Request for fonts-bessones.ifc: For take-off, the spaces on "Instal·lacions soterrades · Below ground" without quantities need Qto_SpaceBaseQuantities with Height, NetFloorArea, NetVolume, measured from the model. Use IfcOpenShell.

First a look at what the model holds.

```python
import ifcopenshell
import ifcopenshell.util.element
import ifcopenshell.util.unit

model = ifcopenshell.open("fonts-bessones.ifc")
print(model.schema)
for unit_type in ("LENGTHUNIT", "AREAUNIT", "VOLUMEUNIT"):
    print(unit_type, ifcopenshell.util.unit.calculate_unit_scale(model, unit_type))
storey = next(s for s in model.by_type("IfcBuildingStorey") if s.Name == "Instal·lacions soterrades · Below ground")
spaces = [e for e in ifcopenshell.util.element.get_decomposition(storey) if e.is_a("IfcSpace")]
for e in sorted(spaces, key=lambda e: e.id()):
    print(e.id(), e.is_a(), e.Name, list(ifcopenshell.util.element.get_psets(e, qtos_only=True)), sep=" | ")
```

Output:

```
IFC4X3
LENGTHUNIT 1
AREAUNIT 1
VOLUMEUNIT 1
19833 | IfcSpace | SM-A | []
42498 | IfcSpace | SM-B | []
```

```python
import ifcopenshell
import ifcopenshell.api.pset
import ifcopenshell.geom
import ifcopenshell.util.element
import ifcopenshell.util.shape
import ifcopenshell.util.unit

model = ifcopenshell.open("fonts-bessones.ifc")
unit_scale = ifcopenshell.util.unit.calculate_unit_scale(model)
area_scale = ifcopenshell.util.unit.calculate_unit_scale(model, "AREAUNIT")
volume_scale = ifcopenshell.util.unit.calculate_unit_scale(model, "VOLUMEUNIT")
settings = ifcopenshell.geom.settings()

storey = next(s for s in model.by_type("IfcBuildingStorey") if s.Name == "Instal·lacions soterrades · Below ground")
spaces = [e for e in ifcopenshell.util.element.get_decomposition(storey) if e.is_a("IfcSpace")]

for e in sorted(spaces, key=lambda e: e.id()):
    if ifcopenshell.util.element.get_psets(e, qtos_only=True, should_inherit=False):
        continue
    # Geometry comes back in metres, in the element's own axes.
    shape = ifcopenshell.geom.create_shape(settings, e)
    values = {
        "Height": ifcopenshell.util.shape.get_z(shape.geometry) / unit_scale,
        "NetFloorArea": ifcopenshell.util.shape.get_footprint_area(shape.geometry) / area_scale,
        "NetVolume": ifcopenshell.util.shape.get_volume(shape.geometry) / volume_scale,
    }
    qto = ifcopenshell.api.pset.add_qto(model, product=e, name="Qto_SpaceBaseQuantities")
    ifcopenshell.api.pset.edit_qto(model, qto=qto, properties=values)
    print(e.id(), {k: round(v, 3) for k, v in values.items()})

model.write("fonts-bessones_edited.ifc")
```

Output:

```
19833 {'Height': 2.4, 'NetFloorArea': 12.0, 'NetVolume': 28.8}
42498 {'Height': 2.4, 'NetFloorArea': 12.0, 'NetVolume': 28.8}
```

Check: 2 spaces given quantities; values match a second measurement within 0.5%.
